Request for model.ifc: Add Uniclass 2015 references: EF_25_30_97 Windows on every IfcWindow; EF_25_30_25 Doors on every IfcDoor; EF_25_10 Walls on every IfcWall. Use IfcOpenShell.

First a look at what the model holds.

```python
import ifcopenshell

model = ifcopenshell.open("model.ifc")
print(model.schema)
print("classifications:", [c.Name for c in model.by_type("IfcClassification")])
for ifc_class in ("IfcDoor", "IfcRoof", "IfcStair", "IfcWall", "IfcWindow"):
    print(ifc_class, len(model.by_type(ifc_class)))
```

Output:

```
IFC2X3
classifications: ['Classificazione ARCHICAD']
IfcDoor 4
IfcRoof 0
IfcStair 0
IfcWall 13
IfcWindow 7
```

```python
import ifcopenshell
import ifcopenshell.api.classification

model = ifcopenshell.open("model.ifc")

# IFC2X3 requires Source and Edition and has no link from the project to the system.
system = model.create_entity("IfcClassification", Source="NBS", Edition="2015", Name="Uniclass 2015")

codes = {
    "IfcWindow": ("EF_25_30_97", "Windows"),
    "IfcDoor": ("EF_25_30_25", "Doors"),
    "IfcWall": ("EF_25_10", "Walls"),
}
for ifc_class, (code, name) in codes.items():
    products = model.by_type(ifc_class)
    ifcopenshell.api.classification.add_reference(
        model, products=products, classification=system, identification=code, name=name
    )
    print(code, len(products))

model.write("model_edited.ifc")
```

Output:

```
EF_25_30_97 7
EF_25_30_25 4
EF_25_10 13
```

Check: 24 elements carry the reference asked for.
